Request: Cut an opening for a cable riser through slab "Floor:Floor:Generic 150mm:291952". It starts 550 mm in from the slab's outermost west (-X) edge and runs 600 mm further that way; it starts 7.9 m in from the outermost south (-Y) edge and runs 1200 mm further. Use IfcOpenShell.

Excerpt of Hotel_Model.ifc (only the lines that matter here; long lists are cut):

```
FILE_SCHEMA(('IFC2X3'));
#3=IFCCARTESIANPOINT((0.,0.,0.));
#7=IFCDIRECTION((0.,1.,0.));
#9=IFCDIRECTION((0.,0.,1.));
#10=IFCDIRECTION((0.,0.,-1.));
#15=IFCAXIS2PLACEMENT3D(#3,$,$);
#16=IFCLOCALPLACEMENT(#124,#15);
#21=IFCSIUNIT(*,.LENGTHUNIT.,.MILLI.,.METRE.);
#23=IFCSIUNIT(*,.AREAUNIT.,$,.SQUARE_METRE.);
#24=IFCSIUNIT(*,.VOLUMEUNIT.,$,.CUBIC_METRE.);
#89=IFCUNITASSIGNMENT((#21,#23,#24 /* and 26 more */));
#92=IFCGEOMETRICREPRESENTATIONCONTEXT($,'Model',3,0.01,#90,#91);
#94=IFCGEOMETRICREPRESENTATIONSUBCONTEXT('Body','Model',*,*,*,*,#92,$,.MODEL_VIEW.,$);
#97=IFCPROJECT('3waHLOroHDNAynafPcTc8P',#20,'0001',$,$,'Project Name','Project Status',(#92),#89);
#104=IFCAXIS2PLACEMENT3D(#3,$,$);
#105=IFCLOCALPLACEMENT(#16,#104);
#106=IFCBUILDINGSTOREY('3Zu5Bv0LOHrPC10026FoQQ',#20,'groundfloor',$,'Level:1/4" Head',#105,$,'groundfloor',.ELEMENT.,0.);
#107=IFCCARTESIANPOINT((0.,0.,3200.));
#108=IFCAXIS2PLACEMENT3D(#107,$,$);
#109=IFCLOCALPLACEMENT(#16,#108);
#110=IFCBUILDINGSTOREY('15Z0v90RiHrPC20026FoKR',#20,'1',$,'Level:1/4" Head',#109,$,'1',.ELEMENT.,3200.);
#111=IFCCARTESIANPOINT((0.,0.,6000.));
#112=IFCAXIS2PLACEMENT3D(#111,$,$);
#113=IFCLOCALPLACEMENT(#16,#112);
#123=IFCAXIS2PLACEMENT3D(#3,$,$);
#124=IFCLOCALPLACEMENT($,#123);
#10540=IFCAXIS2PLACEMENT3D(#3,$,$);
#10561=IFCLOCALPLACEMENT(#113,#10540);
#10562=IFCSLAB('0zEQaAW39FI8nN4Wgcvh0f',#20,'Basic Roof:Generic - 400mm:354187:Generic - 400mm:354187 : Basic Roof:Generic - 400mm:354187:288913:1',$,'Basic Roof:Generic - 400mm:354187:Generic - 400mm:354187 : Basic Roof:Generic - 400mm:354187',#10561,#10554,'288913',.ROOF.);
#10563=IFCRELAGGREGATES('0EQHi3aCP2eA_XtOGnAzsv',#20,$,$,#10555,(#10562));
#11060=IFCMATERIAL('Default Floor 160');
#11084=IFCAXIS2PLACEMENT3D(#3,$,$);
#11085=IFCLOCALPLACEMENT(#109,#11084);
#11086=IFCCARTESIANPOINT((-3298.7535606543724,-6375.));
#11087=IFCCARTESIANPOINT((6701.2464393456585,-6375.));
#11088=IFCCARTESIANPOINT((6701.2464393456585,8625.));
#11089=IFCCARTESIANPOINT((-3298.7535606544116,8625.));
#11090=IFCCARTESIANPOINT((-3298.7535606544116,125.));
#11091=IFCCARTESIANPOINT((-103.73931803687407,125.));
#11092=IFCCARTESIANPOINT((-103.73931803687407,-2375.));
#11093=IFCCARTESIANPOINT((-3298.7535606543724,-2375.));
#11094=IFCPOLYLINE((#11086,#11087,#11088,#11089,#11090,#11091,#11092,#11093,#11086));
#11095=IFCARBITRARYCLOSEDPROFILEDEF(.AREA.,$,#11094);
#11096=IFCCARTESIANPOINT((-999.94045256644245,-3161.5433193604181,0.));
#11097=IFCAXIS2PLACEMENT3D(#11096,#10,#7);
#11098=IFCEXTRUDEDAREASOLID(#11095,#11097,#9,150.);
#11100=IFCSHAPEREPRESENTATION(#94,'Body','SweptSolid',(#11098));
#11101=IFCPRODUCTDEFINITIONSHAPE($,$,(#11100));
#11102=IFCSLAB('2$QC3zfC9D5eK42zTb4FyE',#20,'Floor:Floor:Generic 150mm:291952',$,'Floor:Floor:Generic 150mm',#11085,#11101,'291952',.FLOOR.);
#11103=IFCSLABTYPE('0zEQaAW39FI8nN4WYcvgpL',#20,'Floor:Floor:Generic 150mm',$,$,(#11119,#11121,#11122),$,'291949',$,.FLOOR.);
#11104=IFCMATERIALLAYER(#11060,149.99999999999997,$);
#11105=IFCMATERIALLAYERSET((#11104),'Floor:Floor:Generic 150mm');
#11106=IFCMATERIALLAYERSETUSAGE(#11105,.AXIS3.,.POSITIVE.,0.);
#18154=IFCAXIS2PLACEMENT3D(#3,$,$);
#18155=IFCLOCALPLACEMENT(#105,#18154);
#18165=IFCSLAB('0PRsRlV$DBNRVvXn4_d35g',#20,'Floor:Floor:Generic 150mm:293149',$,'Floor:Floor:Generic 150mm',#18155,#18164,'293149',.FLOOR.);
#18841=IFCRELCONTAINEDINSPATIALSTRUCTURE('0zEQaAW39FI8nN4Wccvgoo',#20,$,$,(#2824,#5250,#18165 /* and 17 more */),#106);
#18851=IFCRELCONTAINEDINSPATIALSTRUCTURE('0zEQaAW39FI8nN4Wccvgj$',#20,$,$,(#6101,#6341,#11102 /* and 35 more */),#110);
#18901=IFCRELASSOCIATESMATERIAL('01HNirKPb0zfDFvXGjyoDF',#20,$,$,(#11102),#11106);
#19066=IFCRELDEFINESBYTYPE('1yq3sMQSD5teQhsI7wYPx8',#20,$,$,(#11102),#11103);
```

```python
import numpy as np
import ifcopenshell
import ifcopenshell.api.feature
import ifcopenshell.api.geometry
import ifcopenshell.api.root
import ifcopenshell.geom
import ifcopenshell.util.placement
import ifcopenshell.util.representation
import ifcopenshell.util.shape
import ifcopenshell.util.unit

model = ifcopenshell.open("Hotel_Model.ifc")
unit_scale = ifcopenshell.util.unit.calculate_unit_scale(model)
settings = ifcopenshell.geom.settings()


def volume(element):
    """Net volume in cubic metres, openings subtracted."""
    shape = ifcopenshell.geom.create_shape(settings, element)
    return ifcopenshell.util.shape.get_volume(shape.geometry)


slab = model.by_guid("2$QC3zfC9D5eK42zTb4FyE")
before = volume(slab)

# Extent in the slab's own axes, in metres. The edges named are its -X and -Y sides.
slab_shape = ifcopenshell.geom.create_shape(settings, slab)
vertices = ifcopenshell.util.shape.get_vertices(slab_shape.geometry)
x_min, y_min, bottom = vertices.min(axis=0)
top = vertices[:, 2].max()

opening = ifcopenshell.api.root.create_entity(model, ifc_class="IfcOpeningElement", name="Cable riser opening")
context = ifcopenshell.util.representation.get_context(model, "Model", "Body", "MODEL_VIEW")
width, depth = 0.6, 1.2
outline = [(0.0, 0.0), (width, 0.0), (width, depth), (0.0, depth), (0.0, 0.0)]
# Overshoot both faces by 50 mm so the cut is clean.
shape = ifcopenshell.api.geometry.add_slab_representation(
    model, context=context, depth=top - bottom + 0.1, polyline=outline
)
ifcopenshell.api.geometry.assign_representation(model, product=opening, representation=shape)

matrix = ifcopenshell.util.placement.get_local_placement(slab.ObjectPlacement)
matrix[:, 3] = matrix @ np.append(np.array([x_min + 0.55, y_min + 7.9, bottom - 0.05]) / unit_scale, 1.0)
ifcopenshell.api.geometry.edit_object_placement(model, product=opening, matrix=matrix, is_si=False)
ifcopenshell.api.feature.add_feature(model, feature=opening, element=slab)

after = volume(slab)

print(f"slab volume {before:.3f} -> {after:.3f} m3")

model.write("Hotel_Model_updated.ifc")
```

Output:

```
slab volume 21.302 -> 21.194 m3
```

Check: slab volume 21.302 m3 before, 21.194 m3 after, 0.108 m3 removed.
